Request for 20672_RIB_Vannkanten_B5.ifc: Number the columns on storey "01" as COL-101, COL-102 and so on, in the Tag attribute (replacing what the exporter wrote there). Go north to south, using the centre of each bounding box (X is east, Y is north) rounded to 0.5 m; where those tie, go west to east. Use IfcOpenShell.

First a look at what the model holds.

```python
import ifcopenshell
import ifcopenshell.util.element
import ifcopenshell.util.placement

model = ifcopenshell.open("20672_RIB_Vannkanten_B5.ifc")
print(model.schema)
storey = next(s for s in model.by_type("IfcBuildingStorey") if s.Name == "01")
columns = [e for e in ifcopenshell.util.element.get_decomposition(storey) if e.is_a("IfcColumn")]
for e in sorted(columns, key=lambda e: e.id()):
    origin = ifcopenshell.util.placement.get_local_placement(e.ObjectPlacement)[:3, 3]
    print(e.id(), e.Tag, e.Name, origin.round(2) + 0.0, sep=" | ")
```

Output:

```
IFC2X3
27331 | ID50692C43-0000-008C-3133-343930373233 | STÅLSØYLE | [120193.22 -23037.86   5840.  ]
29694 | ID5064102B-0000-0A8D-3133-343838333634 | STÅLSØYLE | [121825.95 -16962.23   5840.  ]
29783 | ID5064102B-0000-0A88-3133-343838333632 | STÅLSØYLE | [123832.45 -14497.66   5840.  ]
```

```python
import ifcopenshell
import ifcopenshell.geom
import ifcopenshell.util.element
import ifcopenshell.util.shape

model = ifcopenshell.open("20672_RIB_Vannkanten_B5.ifc")
settings = ifcopenshell.geom.settings()
settings.set("use-world-coords", True)


def centre(element):
    shape = ifcopenshell.geom.create_shape(settings, element)
    return ifcopenshell.util.shape.get_bbox_centroid(shape.geometry)


storey = next(s for s in model.by_type("IfcBuildingStorey") if s.Name == "01")
columns = [e for e in ifcopenshell.util.element.get_decomposition(storey) if e.is_a("IfcColumn")]

# Insertion points can sit at a corner or the storey origin, so sort by the geometry (in metres).
centres = {e: centre(e) for e in columns}
columns.sort(key=lambda e: (-round(centres[e][1] / 0.5), centres[e][0]))

for i, e in enumerate(columns, start=1):
    number = f"COL-1{i:02d}"
    e.Tag = number
    print(e.id(), number)

model.write("20672_RIB_Vannkanten_B5_updated.ifc")
```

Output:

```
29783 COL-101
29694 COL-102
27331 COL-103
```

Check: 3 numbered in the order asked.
